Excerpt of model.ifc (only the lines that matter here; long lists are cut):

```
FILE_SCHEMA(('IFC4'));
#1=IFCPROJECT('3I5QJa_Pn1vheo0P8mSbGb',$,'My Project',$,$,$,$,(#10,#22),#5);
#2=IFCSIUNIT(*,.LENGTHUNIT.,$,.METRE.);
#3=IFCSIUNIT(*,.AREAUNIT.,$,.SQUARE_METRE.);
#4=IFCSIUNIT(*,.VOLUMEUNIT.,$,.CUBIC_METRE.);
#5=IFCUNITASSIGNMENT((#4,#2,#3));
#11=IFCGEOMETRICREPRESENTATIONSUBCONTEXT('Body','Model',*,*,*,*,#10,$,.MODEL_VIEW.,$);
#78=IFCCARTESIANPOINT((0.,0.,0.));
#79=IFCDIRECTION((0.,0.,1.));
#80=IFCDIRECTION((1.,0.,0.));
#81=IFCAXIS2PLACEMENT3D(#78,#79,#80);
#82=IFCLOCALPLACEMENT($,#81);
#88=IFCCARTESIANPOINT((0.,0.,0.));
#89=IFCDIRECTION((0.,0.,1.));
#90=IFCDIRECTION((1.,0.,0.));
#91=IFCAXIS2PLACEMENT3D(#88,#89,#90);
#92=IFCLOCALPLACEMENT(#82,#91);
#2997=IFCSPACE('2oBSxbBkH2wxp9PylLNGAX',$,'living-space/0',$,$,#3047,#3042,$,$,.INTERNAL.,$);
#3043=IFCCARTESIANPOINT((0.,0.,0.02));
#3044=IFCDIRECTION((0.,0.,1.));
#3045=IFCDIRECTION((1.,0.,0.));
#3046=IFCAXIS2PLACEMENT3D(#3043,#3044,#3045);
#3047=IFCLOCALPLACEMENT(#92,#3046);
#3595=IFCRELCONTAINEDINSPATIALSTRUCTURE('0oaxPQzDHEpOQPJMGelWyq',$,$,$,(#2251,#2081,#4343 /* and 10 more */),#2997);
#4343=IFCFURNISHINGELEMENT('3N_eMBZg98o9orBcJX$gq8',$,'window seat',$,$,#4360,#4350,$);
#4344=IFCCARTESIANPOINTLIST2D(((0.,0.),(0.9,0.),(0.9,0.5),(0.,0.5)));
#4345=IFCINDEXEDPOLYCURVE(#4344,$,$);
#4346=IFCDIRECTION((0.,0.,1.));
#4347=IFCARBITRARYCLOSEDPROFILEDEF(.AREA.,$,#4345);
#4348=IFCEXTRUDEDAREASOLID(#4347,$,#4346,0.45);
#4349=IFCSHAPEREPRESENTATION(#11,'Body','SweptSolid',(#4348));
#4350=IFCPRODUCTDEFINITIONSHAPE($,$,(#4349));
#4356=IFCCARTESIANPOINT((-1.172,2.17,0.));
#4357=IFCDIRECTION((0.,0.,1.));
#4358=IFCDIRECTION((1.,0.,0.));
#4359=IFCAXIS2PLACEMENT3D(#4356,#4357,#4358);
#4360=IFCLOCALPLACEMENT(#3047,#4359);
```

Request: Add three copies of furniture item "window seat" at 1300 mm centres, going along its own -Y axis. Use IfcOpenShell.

```python
import ifcopenshell
import ifcopenshell.api.geometry
import ifcopenshell.api.root
import ifcopenshell.util.element
import ifcopenshell.util.placement
import ifcopenshell.util.unit

model = ifcopenshell.open("model.ifc")
unit_scale = ifcopenshell.util.unit.calculate_unit_scale(model)

source = model.by_guid("3N_eMBZg98o9orBcJX$gq8")
base = ifcopenshell.util.placement.get_local_placement(source.ObjectPlacement)
step = -base[:3, 1] * 1.3 / unit_scale

for i in range(1, 4):
    copy = ifcopenshell.api.root.copy_class(model, product=source)
    copy.Representation = ifcopenshell.util.element.copy_deep(
        model, source.Representation, exclude=["IfcGeometricRepresentationContext", "IfcRepresentationMap"]
    )
    matrix = base.copy()
    matrix[:3, 3] += i * step
    print("added at", matrix[:3, 3].round(3) + 0.0)
    ifcopenshell.api.geometry.edit_object_placement(model, product=copy, matrix=matrix, is_si=False)

model.write("model_rev.ifc")
```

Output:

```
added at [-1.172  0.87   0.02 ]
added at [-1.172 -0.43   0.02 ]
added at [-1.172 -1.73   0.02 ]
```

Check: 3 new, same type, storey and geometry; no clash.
